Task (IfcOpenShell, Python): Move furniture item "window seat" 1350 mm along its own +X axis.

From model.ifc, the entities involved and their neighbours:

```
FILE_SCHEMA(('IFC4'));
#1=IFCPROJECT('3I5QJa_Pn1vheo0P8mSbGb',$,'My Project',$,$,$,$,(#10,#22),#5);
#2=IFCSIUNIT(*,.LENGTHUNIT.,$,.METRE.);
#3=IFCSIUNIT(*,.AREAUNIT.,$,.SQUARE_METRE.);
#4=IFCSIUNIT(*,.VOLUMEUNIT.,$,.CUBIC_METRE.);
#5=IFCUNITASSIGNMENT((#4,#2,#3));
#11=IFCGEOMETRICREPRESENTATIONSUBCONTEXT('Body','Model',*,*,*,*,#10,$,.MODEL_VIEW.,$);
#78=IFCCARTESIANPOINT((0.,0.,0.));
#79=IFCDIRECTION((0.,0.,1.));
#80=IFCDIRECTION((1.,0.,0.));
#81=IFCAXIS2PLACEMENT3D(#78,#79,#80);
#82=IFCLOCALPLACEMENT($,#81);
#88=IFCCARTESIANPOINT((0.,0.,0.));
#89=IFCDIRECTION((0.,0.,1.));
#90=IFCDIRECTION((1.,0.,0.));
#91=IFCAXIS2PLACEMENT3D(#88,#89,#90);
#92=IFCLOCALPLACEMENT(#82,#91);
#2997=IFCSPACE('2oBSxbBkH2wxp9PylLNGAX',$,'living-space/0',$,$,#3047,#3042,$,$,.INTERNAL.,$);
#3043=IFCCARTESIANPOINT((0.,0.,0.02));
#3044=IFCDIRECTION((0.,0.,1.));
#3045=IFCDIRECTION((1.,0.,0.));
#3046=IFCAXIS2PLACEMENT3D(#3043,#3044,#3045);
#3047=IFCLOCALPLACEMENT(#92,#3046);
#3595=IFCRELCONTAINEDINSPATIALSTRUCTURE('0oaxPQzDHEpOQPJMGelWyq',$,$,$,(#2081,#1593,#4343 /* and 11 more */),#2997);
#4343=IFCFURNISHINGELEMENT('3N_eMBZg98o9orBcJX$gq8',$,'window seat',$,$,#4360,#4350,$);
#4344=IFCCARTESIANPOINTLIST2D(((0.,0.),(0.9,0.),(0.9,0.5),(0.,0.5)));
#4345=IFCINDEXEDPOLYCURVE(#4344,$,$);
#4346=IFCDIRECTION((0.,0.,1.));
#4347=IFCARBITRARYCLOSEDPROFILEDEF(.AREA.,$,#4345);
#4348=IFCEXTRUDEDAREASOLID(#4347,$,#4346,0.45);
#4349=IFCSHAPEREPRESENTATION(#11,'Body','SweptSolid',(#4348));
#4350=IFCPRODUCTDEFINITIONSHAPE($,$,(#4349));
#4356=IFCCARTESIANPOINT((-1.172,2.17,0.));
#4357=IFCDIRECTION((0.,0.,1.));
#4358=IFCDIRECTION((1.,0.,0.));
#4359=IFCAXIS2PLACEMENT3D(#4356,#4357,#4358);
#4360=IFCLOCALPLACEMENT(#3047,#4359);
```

```python
import ifcopenshell
import ifcopenshell.api.geometry
import ifcopenshell.util.placement
import ifcopenshell.util.unit

model = ifcopenshell.open("model.ifc")
unit_scale = ifcopenshell.util.unit.calculate_unit_scale(model)

item = model.by_guid("3N_eMBZg98o9orBcJX$gq8")
matrix = ifcopenshell.util.placement.get_local_placement(item.ObjectPlacement)
matrix[:3, 3] += matrix[:3, 0] * 1.35 / unit_scale
ifcopenshell.api.geometry.edit_object_placement(model, product=item, matrix=matrix, is_si=False)

print(ifcopenshell.util.placement.get_local_placement(item.ObjectPlacement).round(3) + 0.0)

model.write("model_v2.ifc")
```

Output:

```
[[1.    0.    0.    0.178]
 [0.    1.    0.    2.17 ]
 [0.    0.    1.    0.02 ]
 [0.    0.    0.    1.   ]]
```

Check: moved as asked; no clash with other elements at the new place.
